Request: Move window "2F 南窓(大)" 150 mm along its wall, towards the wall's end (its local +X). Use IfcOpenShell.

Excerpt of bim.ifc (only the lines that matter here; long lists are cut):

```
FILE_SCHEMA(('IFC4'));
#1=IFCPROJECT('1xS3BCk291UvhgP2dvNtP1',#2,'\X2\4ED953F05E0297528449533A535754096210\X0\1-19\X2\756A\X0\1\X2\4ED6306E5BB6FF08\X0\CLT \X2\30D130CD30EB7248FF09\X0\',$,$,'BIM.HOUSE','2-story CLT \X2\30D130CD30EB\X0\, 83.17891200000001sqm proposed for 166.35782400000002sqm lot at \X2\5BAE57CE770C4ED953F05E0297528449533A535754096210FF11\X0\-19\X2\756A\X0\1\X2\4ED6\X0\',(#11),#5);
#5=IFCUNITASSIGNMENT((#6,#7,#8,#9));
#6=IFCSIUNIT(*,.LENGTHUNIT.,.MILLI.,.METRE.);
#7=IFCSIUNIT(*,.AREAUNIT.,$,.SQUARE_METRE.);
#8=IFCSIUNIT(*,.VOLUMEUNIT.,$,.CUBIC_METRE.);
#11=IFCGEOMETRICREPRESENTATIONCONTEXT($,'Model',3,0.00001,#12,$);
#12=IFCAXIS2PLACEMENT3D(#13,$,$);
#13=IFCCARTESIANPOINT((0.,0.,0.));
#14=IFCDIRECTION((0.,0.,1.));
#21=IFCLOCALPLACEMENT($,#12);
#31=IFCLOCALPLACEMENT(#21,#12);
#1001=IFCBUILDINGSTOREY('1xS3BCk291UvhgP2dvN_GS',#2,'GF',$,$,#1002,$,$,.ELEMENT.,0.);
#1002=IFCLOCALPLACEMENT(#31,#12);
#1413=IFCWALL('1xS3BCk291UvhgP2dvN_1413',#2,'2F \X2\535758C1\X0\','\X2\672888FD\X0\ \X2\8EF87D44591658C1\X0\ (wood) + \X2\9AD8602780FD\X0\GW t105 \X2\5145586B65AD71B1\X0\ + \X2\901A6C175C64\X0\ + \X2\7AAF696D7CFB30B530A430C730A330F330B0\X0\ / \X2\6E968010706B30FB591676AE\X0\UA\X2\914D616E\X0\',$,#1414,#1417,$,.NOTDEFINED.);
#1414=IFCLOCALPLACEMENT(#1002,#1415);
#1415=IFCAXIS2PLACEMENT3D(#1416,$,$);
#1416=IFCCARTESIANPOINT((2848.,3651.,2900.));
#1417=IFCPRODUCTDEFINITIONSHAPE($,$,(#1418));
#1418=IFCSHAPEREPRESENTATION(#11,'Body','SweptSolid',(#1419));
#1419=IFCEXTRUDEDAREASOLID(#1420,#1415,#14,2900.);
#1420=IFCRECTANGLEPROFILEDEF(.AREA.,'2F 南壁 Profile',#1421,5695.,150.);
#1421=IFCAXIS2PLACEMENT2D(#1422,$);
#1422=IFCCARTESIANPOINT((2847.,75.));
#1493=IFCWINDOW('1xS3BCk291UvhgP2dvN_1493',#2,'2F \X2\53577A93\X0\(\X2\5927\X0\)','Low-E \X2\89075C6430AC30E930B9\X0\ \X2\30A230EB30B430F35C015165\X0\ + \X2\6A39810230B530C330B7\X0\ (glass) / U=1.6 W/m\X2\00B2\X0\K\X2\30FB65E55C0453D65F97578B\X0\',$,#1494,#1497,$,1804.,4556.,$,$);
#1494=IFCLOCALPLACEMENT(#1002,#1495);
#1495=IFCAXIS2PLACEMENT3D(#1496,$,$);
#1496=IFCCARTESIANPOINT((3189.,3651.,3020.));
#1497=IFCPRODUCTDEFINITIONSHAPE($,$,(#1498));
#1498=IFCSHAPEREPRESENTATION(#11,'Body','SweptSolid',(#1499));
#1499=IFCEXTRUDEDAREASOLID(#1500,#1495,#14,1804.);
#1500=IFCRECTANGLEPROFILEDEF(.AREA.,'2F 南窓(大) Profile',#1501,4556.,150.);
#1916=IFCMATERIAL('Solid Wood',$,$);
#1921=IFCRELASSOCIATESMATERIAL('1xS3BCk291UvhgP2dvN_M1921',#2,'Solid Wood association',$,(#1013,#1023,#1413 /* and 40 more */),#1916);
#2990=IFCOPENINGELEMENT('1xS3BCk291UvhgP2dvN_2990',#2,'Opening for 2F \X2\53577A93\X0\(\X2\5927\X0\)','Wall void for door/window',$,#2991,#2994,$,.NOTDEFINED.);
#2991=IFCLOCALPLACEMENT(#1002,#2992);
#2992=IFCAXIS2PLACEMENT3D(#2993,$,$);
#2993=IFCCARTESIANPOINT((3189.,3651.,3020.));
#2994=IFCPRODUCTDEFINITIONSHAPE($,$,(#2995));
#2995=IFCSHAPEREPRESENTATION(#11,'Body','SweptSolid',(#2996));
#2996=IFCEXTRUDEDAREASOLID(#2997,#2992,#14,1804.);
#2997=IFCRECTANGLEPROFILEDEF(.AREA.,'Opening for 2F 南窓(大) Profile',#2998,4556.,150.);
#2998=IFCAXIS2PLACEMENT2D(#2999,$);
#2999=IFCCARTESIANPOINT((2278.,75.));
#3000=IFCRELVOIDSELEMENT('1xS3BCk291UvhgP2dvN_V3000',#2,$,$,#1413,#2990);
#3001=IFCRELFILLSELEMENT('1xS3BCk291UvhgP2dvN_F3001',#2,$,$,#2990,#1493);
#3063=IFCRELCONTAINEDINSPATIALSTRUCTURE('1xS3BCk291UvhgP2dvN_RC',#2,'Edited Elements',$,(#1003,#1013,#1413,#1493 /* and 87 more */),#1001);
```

```python
import ifcopenshell
import ifcopenshell.api.geometry
import ifcopenshell.util.placement
import ifcopenshell.util.unit

model = ifcopenshell.open("bim.ifc")
unit_scale = ifcopenshell.util.unit.calculate_unit_scale(model)

window = model.by_id(1493)
opening = window.FillsVoids[0].RelatingOpeningElement
wall = opening.VoidsElements[0].RelatingBuildingElement

wall_matrix = ifcopenshell.util.placement.get_local_placement(wall.ObjectPlacement)
shift = wall_matrix[:3, 0] * 0.15 / unit_scale
before = ifcopenshell.util.placement.get_local_placement(window.ObjectPlacement)[:3, 3].copy()

# The window is not placed relative to its opening, so move both.
for product in (opening, window):
    matrix = ifcopenshell.util.placement.get_local_placement(product.ObjectPlacement)
    matrix[:3, 3] += shift
    ifcopenshell.api.geometry.edit_object_placement(model, product=product, matrix=matrix, is_si=False)

after = ifcopenshell.util.placement.get_local_placement(window.ObjectPlacement)[:3, 3]
print("window moved by", (after - before).round(3) + 0.0)

model.write("bim_v2.ifc")
```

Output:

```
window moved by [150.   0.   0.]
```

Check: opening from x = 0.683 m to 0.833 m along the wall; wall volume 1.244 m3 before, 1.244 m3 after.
